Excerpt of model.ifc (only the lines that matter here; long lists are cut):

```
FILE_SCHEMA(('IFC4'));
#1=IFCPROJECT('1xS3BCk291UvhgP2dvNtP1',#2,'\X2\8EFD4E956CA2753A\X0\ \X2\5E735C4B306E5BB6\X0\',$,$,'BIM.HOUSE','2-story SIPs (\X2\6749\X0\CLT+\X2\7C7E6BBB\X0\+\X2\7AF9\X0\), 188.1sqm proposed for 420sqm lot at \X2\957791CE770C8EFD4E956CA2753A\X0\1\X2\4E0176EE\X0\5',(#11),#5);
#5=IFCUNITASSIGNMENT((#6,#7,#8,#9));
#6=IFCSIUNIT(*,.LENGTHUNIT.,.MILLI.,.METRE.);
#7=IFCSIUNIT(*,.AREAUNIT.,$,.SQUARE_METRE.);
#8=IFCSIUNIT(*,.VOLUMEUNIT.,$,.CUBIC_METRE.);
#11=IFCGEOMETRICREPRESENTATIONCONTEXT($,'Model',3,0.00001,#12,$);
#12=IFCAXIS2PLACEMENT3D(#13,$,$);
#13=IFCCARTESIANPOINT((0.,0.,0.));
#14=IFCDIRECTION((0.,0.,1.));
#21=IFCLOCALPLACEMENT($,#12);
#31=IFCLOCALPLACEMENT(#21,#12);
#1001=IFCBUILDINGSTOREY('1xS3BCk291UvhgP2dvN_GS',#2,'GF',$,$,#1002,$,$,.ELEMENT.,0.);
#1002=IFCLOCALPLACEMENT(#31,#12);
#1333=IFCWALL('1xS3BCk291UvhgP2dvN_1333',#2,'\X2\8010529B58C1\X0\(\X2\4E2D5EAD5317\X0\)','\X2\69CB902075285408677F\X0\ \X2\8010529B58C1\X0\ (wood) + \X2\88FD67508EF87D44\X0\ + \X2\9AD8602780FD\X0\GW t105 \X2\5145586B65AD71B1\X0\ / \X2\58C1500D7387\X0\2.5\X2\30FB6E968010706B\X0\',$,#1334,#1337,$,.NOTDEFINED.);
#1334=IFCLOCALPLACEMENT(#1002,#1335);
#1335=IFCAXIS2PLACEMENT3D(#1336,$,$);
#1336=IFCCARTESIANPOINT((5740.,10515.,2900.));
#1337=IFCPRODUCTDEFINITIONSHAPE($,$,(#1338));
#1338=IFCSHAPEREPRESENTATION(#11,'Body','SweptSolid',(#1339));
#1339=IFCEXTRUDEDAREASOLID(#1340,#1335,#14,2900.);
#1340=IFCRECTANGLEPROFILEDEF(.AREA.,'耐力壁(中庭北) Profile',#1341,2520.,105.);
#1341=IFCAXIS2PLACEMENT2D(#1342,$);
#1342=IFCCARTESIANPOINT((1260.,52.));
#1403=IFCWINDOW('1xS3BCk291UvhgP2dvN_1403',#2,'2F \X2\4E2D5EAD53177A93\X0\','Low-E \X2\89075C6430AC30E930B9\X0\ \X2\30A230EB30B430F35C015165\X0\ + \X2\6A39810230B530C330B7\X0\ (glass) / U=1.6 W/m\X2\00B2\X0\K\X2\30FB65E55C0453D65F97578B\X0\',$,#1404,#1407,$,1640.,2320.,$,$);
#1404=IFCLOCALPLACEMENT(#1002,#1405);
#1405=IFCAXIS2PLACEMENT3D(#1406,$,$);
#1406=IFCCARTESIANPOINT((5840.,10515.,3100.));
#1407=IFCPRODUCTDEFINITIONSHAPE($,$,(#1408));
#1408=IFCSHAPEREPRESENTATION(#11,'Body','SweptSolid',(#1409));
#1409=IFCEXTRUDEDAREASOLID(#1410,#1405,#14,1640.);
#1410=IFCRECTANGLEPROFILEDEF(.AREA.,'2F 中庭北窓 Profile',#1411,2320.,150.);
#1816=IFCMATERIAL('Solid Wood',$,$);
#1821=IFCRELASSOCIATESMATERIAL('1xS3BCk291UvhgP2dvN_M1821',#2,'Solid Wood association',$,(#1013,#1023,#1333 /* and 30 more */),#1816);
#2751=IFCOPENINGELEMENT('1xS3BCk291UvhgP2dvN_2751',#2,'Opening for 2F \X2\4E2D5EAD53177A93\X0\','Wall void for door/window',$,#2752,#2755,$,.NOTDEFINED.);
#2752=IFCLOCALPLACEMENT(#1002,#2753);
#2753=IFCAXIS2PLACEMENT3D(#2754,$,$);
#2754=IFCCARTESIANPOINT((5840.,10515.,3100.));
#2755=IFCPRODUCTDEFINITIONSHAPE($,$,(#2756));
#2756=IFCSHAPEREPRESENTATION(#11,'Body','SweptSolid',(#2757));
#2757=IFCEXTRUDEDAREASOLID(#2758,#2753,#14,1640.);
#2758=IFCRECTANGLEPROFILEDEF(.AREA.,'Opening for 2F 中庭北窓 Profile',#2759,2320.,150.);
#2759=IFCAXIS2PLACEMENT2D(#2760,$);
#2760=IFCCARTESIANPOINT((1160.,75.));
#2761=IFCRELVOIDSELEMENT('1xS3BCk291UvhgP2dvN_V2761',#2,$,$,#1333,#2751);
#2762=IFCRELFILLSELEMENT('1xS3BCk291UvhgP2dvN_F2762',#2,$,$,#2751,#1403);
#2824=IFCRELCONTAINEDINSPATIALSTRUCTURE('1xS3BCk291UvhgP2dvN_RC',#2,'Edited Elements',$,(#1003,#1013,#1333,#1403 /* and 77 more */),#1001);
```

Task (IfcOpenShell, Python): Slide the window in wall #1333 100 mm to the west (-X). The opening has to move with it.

```python
import ifcopenshell
import ifcopenshell.api.geometry
import ifcopenshell.util.placement
import ifcopenshell.util.unit

model = ifcopenshell.open("model.ifc")
unit_scale = ifcopenshell.util.unit.calculate_unit_scale(model)

window = model.by_guid("1xS3BCk291UvhgP2dvN_1403")
opening = window.FillsVoids[0].RelatingOpeningElement
wall = opening.VoidsElements[0].RelatingBuildingElement

wall_matrix = ifcopenshell.util.placement.get_local_placement(wall.ObjectPlacement)
shift = wall_matrix[:3, 0] * -0.1 / unit_scale
before = ifcopenshell.util.placement.get_local_placement(window.ObjectPlacement)[:3, 3].copy()

# The window is not placed relative to its opening, so move both.
for product in (opening, window):
    matrix = ifcopenshell.util.placement.get_local_placement(product.ObjectPlacement)
    matrix[:3, 3] += shift
    ifcopenshell.api.geometry.edit_object_placement(model, product=product, matrix=matrix, is_si=False)

after = ifcopenshell.util.placement.get_local_placement(window.ObjectPlacement)[:3, 3]
print("window moved by", (after - before).round(3) + 0.0)

model.write("model_edited.ifc")
```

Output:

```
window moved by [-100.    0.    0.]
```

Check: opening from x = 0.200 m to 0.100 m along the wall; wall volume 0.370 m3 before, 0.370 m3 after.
